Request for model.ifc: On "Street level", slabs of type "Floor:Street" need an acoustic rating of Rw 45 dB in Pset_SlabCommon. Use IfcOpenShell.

First a look at what the model holds.

```python
import ifcopenshell
import ifcopenshell.util.element

model = ifcopenshell.open("model.ifc")
print(model.schema)
storey = next(s for s in model.by_type("IfcBuildingStorey") if s.Name == "Street level")
slabs = [e for e in ifcopenshell.util.element.get_decomposition(storey) if e.is_a("IfcSlab")]
seen = {}
for e in slabs:
    element_type = ifcopenshell.util.element.get_type(e)
    key = (element_type.Name if element_type != e and element_type else None, ifcopenshell.util.element.get_pset(e, "Pset_SlabCommon", "AcousticRating"))
    seen[key] = seen.get(key, 0) + 1
for (name, value), count in sorted(seen.items(), key=str):
    print(count, "x", name, "|", value)
```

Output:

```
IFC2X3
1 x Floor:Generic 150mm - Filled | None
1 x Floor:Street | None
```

```python
import ifcopenshell
import ifcopenshell.api.pset
import ifcopenshell.util.element

model = ifcopenshell.open("model.ifc")

storey = next(s for s in model.by_type("IfcBuildingStorey") if s.Name == "Street level")
slabs = [e for e in ifcopenshell.util.element.get_decomposition(storey) if e.is_a("IfcSlab")]

count = 0
for e in slabs:
    element_type = ifcopenshell.util.element.get_type(e)
    if element_type in (None, e) or element_type.Name != "Floor:Street":
        continue
    # add_pset returns the element's existing set when there is one.
    pset = ifcopenshell.api.pset.add_pset(model, product=e, name="Pset_SlabCommon")
    ifcopenshell.api.pset.edit_pset(model, pset=pset, properties={"AcousticRating": "Rw 45 dB"})
    count += 1

print(count, "slabs updated")

model.write("model_updated.ifc")
```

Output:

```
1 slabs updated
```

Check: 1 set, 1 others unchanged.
